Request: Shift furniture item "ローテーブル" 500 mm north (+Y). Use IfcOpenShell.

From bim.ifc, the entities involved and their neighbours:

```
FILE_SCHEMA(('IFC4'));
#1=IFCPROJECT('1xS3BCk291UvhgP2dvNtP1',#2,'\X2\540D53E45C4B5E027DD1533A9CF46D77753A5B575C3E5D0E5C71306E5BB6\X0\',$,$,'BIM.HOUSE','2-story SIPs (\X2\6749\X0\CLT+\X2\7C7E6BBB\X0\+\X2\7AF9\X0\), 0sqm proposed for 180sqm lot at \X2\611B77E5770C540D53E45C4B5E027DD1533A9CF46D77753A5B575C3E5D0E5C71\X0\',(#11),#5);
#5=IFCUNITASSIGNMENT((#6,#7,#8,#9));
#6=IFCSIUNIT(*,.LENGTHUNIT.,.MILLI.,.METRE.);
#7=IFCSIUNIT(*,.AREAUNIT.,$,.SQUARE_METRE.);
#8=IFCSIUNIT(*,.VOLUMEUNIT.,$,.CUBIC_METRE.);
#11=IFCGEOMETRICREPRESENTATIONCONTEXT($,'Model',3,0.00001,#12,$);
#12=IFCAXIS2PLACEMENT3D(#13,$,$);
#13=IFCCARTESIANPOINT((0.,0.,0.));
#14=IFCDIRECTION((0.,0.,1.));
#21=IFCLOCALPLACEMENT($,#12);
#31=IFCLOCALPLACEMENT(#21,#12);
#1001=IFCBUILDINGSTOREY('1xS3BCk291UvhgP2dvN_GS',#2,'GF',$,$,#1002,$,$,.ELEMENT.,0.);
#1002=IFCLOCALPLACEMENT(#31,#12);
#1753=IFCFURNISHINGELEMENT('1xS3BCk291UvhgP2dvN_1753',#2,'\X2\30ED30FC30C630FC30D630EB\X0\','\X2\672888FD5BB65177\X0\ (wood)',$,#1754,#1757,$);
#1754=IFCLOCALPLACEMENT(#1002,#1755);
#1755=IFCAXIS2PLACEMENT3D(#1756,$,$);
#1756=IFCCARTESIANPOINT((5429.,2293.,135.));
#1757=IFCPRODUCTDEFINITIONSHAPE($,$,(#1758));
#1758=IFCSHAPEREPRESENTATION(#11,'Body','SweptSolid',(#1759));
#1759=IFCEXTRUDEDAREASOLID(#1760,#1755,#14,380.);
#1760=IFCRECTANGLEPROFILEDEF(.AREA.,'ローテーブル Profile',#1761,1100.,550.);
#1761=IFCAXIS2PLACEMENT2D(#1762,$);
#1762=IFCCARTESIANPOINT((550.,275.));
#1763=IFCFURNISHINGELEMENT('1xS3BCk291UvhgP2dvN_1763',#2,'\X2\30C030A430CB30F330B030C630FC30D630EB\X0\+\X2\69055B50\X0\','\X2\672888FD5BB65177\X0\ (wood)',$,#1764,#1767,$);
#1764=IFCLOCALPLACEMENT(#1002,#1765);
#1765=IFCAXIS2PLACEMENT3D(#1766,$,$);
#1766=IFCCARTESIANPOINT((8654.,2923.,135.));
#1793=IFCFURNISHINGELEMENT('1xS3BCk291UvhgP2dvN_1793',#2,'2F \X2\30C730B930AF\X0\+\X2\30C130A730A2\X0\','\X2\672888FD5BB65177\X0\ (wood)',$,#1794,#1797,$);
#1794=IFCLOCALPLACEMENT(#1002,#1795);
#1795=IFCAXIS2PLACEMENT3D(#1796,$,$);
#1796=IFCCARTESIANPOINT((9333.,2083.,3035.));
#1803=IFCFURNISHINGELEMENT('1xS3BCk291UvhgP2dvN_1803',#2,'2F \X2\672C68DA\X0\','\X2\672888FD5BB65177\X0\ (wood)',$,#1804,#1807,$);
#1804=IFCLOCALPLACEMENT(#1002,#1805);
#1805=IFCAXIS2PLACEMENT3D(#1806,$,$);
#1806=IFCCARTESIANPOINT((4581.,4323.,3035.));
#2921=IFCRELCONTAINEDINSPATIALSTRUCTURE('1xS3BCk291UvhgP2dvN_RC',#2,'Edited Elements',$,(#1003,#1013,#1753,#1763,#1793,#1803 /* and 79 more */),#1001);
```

```python
import ifcopenshell
import ifcopenshell.api.geometry
import ifcopenshell.util.placement
import ifcopenshell.util.unit

model = ifcopenshell.open("bim.ifc")
unit_scale = ifcopenshell.util.unit.calculate_unit_scale(model)

item = model.by_guid("1xS3BCk291UvhgP2dvN_1753")
matrix = ifcopenshell.util.placement.get_local_placement(item.ObjectPlacement)
matrix[1, 3] += 0.5 / unit_scale
ifcopenshell.api.geometry.edit_object_placement(model, product=item, matrix=matrix, is_si=False)

print(ifcopenshell.util.placement.get_local_placement(item.ObjectPlacement).round(3) + 0.0)

model.write("bim_v2.ifc")
```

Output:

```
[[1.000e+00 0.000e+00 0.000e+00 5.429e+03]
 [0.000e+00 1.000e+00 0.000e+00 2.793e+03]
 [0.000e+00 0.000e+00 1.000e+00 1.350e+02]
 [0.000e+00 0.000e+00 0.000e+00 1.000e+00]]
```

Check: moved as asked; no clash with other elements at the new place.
